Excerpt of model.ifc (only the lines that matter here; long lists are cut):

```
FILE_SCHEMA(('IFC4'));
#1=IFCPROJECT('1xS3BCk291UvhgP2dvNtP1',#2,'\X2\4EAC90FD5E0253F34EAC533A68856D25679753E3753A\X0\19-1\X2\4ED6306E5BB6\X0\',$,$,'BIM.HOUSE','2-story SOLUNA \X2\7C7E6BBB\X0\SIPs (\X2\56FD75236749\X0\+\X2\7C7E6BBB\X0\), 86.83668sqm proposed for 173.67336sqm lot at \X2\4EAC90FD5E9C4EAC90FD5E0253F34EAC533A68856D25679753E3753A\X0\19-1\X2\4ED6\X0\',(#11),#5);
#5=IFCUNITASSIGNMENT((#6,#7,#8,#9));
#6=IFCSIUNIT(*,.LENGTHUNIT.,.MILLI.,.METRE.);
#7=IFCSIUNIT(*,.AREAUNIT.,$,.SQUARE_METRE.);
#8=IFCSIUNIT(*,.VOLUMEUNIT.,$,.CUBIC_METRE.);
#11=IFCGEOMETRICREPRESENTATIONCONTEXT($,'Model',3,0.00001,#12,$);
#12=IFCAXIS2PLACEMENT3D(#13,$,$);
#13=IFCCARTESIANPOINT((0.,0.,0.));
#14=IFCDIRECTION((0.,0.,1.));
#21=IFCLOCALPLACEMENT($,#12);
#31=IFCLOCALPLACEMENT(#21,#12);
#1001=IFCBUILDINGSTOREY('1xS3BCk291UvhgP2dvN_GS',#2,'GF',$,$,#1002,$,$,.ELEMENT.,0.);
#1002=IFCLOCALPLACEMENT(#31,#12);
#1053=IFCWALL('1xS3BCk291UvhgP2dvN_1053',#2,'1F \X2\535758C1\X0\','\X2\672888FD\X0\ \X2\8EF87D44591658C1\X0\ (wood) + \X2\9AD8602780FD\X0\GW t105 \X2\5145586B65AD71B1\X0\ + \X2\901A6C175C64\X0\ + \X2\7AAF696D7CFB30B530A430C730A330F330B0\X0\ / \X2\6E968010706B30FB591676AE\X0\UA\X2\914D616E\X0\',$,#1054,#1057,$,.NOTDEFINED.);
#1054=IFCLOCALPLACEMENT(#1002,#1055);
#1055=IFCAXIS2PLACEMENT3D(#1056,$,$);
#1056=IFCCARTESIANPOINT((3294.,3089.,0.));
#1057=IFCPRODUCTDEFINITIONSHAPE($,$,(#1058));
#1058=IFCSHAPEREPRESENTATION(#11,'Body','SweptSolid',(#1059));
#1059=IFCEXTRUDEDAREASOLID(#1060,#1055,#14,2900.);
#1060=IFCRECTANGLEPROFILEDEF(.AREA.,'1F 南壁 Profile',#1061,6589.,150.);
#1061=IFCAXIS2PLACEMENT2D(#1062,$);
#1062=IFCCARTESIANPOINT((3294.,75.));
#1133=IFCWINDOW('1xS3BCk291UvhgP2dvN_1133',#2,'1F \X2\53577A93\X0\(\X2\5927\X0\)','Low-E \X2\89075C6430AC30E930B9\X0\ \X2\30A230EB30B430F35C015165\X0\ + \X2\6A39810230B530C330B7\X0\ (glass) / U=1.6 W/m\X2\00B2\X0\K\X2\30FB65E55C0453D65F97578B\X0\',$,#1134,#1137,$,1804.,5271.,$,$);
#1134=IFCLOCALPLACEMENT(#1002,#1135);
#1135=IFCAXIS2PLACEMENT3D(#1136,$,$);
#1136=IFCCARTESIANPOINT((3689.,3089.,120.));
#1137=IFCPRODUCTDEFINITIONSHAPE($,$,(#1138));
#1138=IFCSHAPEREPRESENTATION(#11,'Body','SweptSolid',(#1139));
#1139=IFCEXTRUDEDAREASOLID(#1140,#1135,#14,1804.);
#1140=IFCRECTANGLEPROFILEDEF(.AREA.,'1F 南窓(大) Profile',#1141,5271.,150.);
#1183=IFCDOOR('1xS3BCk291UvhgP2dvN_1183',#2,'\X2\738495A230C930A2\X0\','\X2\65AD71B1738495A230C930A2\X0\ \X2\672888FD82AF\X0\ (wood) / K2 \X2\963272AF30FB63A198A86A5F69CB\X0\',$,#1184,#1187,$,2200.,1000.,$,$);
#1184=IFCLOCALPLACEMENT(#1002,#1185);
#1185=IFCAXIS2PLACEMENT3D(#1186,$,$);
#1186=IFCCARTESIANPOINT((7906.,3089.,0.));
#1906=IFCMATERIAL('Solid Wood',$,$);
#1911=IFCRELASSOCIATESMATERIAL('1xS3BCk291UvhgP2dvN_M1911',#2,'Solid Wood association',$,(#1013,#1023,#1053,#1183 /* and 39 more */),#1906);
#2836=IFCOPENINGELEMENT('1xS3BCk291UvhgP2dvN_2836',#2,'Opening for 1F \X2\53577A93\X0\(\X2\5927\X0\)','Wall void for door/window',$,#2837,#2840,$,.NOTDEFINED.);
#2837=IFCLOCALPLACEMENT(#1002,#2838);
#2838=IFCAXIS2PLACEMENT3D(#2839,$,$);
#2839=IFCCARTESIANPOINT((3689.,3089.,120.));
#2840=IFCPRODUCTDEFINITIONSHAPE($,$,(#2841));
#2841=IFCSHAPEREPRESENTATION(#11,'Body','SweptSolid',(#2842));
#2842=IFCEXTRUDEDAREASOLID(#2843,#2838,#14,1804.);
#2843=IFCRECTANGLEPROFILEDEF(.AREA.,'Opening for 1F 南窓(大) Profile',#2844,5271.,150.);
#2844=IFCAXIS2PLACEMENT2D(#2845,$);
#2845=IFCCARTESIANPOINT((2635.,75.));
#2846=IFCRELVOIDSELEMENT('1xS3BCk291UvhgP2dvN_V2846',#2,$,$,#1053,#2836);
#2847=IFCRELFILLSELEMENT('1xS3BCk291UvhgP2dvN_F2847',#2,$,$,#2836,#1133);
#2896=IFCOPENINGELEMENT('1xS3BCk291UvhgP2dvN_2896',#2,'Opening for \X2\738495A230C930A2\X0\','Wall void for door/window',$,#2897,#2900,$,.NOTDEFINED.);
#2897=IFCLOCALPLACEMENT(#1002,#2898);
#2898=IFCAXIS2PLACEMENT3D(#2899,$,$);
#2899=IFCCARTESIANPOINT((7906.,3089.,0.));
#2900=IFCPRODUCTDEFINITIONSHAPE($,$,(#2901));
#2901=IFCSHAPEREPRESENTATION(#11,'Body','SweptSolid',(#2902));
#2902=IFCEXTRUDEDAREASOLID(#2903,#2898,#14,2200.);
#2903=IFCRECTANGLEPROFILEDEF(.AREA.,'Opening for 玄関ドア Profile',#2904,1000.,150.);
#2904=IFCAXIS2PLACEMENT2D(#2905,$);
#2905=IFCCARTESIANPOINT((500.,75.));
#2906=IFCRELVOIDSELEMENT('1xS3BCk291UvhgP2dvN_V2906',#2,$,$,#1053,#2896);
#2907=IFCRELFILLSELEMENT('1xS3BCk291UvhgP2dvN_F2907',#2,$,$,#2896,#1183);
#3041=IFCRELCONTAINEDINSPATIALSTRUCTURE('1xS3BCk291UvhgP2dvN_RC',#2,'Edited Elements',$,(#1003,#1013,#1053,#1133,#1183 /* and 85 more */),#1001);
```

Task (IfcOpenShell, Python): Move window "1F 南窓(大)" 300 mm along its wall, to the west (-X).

```python
import ifcopenshell
import ifcopenshell.api.geometry
import ifcopenshell.util.placement

model = ifcopenshell.open("model.ifc")

window = model.by_guid("1xS3BCk291UvhgP2dvN_1133")
opening = window.FillsVoids[0].RelatingOpeningElement
wall = opening.VoidsElements[0].RelatingBuildingElement

wall_matrix = ifcopenshell.util.placement.get_local_placement(wall.ObjectPlacement)
shift = wall_matrix[:3, 0] * -300.0
before = ifcopenshell.util.placement.get_local_placement(window.ObjectPlacement)[:3, 3].copy()

# The window is not placed relative to its opening, so move both.
for product in (opening, window):
    matrix = ifcopenshell.util.placement.get_local_placement(product.ObjectPlacement)
    matrix[:3, 3] += shift
    ifcopenshell.api.geometry.edit_object_placement(model, product=product, matrix=matrix, is_si=False)

after = ifcopenshell.util.placement.get_local_placement(window.ObjectPlacement)[:3, 3]
print("window moved by", (after - before).round(3) + 0.0)

model.write("model_rev.ifc")
```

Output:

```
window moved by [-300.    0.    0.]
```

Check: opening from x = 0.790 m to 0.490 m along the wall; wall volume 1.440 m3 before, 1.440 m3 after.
